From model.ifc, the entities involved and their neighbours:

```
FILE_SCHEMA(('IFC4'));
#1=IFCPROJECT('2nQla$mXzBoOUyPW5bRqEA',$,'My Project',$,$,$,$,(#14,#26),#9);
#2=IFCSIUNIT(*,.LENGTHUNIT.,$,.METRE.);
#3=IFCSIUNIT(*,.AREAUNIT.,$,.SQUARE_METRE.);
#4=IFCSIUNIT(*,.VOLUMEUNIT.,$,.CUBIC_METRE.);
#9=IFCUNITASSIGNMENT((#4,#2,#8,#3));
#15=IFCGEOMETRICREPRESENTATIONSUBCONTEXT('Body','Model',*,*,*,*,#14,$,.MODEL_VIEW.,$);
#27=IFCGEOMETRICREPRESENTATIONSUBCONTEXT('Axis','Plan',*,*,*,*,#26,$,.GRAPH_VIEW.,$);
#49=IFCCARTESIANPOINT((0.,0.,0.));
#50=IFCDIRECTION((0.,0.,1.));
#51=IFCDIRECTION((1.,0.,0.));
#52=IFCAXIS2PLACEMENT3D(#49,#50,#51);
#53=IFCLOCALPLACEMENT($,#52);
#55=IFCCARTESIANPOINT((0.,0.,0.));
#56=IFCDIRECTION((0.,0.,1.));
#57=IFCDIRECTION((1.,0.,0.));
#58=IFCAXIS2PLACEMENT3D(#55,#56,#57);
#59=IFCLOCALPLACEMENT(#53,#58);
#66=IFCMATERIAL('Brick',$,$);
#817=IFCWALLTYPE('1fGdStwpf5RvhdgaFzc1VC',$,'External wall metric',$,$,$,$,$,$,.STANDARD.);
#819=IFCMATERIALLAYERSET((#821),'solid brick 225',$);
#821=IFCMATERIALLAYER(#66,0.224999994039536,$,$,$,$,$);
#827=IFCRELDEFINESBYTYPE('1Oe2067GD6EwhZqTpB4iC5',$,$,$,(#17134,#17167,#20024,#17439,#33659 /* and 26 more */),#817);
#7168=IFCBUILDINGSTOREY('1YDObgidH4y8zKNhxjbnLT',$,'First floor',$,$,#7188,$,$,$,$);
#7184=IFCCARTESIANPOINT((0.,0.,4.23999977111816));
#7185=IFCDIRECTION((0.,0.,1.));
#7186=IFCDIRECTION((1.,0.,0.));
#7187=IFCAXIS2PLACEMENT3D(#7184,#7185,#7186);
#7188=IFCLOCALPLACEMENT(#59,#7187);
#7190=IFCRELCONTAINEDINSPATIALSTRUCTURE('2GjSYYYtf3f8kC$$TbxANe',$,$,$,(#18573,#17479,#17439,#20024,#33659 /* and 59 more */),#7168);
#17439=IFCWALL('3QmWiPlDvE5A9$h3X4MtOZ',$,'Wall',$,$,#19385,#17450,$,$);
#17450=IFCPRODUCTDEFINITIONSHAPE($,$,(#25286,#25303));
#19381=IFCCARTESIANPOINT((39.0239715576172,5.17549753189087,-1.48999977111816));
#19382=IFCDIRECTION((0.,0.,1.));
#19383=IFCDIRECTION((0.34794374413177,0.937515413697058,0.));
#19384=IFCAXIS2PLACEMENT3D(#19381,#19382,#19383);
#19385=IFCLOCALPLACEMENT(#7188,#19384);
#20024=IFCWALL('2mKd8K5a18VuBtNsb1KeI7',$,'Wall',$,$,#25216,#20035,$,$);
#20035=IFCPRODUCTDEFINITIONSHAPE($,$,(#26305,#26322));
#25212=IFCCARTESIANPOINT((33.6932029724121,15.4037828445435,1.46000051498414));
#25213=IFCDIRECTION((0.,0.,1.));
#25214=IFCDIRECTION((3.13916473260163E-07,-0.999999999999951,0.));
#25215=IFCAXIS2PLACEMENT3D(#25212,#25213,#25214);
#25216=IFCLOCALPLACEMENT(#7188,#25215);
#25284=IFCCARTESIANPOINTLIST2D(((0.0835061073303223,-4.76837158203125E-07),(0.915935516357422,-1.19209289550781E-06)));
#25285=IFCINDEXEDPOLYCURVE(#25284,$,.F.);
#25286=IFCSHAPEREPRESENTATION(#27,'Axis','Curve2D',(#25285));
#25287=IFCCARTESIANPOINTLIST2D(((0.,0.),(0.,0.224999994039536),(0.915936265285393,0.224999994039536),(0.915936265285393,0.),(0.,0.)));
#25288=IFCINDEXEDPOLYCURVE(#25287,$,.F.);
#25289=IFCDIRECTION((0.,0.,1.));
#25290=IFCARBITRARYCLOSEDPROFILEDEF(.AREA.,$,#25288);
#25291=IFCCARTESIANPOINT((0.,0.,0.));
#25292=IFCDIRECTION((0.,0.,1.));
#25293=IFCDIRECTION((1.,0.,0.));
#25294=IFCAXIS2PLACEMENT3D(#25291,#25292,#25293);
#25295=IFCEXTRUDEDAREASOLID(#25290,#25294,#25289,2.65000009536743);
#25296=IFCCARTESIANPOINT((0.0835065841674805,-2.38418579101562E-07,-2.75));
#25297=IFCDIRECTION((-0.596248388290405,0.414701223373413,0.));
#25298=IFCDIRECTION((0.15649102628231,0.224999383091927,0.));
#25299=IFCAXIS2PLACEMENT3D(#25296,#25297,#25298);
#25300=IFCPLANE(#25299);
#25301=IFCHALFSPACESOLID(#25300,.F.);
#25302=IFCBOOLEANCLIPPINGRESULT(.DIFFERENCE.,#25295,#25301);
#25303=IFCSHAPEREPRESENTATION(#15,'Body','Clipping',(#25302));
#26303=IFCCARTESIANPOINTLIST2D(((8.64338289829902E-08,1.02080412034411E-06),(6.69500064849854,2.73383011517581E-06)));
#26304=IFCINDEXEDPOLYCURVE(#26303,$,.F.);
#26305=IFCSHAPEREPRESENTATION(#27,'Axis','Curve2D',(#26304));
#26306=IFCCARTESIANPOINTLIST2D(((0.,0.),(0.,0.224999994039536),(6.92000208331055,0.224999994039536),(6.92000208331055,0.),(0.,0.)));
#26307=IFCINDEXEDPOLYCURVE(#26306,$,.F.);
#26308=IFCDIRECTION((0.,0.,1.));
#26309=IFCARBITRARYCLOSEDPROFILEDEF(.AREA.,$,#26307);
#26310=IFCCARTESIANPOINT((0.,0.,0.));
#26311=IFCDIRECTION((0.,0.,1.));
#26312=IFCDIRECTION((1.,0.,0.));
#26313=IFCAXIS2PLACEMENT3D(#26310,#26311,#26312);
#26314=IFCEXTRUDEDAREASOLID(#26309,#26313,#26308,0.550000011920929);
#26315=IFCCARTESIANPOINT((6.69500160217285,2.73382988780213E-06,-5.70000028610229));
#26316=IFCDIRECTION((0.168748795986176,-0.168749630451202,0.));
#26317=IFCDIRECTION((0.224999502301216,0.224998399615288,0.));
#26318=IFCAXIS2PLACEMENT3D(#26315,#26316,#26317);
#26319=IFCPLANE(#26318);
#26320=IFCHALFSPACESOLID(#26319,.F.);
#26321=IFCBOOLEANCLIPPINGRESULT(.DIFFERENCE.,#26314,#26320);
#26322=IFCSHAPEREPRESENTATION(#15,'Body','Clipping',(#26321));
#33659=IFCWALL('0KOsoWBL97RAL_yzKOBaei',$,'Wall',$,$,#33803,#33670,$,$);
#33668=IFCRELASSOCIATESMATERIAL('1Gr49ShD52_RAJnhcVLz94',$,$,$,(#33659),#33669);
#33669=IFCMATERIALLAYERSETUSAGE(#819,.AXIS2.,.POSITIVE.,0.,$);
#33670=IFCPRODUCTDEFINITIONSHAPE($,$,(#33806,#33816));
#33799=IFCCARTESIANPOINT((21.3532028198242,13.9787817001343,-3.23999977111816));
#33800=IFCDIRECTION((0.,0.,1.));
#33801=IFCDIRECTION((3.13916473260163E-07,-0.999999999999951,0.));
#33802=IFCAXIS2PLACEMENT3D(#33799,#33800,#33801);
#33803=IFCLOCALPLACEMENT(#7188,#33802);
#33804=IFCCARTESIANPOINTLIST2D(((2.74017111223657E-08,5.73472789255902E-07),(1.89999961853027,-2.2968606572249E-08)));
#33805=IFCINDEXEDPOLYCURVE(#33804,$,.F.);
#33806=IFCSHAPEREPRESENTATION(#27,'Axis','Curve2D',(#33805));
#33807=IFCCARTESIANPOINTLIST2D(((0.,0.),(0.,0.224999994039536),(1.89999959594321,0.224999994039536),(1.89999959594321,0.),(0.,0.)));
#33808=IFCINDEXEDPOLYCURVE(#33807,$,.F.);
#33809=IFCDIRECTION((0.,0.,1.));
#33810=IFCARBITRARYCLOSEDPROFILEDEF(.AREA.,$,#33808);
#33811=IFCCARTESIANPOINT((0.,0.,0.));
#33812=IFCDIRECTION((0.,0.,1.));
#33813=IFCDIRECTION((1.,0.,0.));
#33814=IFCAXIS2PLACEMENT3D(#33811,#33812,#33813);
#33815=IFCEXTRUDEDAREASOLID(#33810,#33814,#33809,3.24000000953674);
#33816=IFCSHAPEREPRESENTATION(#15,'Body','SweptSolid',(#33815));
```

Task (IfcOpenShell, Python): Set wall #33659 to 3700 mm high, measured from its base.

```python
import ifcopenshell
import ifcopenshell.geom
import ifcopenshell.util.representation
import ifcopenshell.util.shape
import ifcopenshell.util.unit

model = ifcopenshell.open("model.ifc")
unit_scale = ifcopenshell.util.unit.calculate_unit_scale(model)
settings = ifcopenshell.geom.settings()


def volume(element):
    """Net volume in cubic metres, openings subtracted."""
    shape = ifcopenshell.geom.create_shape(settings, element)
    return ifcopenshell.util.shape.get_volume(shape.geometry)


wall = model.by_id(33659)
before = volume(wall)

body = ifcopenshell.util.representation.get_representation(wall, "Model", "Body")
solid = body.Items[0]
old_height = solid.Depth
solid.Depth = 3.7 / unit_scale
after = volume(wall)

print(f"height {old_height:g} -> {solid.Depth:g}, volume {before:.3f} -> {after:.3f} m3")

model.write("model_v2.ifc")
```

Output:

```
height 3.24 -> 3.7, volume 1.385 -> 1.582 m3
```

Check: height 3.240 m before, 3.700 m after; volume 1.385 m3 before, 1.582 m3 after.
